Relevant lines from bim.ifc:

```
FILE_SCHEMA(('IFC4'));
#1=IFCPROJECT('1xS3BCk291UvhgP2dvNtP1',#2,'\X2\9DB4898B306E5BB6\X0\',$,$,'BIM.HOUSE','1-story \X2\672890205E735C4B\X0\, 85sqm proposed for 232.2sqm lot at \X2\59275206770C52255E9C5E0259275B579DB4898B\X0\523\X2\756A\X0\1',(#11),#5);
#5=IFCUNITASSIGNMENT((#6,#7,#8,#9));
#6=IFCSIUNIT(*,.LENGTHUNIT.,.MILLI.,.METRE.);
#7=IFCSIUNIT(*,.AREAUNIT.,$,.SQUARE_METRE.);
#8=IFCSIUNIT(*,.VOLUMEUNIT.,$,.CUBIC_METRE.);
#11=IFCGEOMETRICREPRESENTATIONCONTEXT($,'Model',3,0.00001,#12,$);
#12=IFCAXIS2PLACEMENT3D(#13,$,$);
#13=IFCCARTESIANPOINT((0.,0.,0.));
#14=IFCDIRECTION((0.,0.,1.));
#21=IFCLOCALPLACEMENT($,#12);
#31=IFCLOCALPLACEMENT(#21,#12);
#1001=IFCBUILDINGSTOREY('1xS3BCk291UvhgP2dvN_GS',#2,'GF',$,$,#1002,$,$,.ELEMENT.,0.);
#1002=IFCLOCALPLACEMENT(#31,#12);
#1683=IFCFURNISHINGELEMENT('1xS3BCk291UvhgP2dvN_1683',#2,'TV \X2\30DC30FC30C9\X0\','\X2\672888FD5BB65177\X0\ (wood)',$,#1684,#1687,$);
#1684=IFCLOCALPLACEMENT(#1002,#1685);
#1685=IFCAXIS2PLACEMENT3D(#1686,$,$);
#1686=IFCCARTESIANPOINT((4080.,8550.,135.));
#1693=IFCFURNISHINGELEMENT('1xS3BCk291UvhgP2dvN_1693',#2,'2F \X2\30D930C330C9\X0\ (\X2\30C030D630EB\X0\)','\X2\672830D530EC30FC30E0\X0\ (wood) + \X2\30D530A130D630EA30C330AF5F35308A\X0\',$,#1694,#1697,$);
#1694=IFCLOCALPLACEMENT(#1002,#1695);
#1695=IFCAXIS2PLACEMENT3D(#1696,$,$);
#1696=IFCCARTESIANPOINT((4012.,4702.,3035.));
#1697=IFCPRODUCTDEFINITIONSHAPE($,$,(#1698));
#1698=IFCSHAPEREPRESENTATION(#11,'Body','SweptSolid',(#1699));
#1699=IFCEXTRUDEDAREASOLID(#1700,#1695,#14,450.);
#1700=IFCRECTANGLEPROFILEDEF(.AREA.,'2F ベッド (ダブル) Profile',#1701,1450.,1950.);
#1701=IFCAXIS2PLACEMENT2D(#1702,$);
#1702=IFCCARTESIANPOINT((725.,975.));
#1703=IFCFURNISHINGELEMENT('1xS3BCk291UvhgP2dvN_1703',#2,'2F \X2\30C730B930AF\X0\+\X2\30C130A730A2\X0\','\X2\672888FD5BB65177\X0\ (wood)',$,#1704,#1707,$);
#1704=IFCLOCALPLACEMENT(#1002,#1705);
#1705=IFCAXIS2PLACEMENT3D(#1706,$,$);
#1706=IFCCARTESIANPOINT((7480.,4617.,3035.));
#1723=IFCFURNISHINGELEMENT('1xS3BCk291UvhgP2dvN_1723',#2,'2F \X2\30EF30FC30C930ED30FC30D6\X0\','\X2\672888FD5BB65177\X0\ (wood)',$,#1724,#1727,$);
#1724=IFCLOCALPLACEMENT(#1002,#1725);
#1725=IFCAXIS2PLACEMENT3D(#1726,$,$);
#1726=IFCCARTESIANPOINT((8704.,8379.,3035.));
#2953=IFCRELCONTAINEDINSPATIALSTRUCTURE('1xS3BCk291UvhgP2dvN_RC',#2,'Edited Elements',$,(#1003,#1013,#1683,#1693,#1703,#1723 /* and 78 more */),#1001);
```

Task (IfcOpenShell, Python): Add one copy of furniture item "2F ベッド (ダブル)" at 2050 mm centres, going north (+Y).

```python
import numpy as np
import ifcopenshell
import ifcopenshell.api.geometry
import ifcopenshell.api.root
import ifcopenshell.util.element
import ifcopenshell.util.placement
import ifcopenshell.util.unit

model = ifcopenshell.open("bim.ifc")
unit_scale = ifcopenshell.util.unit.calculate_unit_scale(model)


def reuse_history(source, copy):
    """copy_class also copies each property set's owner history, people and application; keep the originals."""
    for rel in copy.IsDefinedBy:
        if rel.is_a("IfcRelDefinesByProperties") and (history := rel.RelatingPropertyDefinition.OwnerHistory):
            rel.RelatingPropertyDefinition.OwnerHistory = source.OwnerHistory
            ifcopenshell.util.element.remove_deep2(model, history)


source = model.by_id(1693)
base = ifcopenshell.util.placement.get_local_placement(source.ObjectPlacement)
step = np.array([0.0, 1.0, 0.0]) * 2.05 / unit_scale

for i in range(1, 2):
    copy = ifcopenshell.api.root.copy_class(model, product=source)
    copy.Representation = ifcopenshell.util.element.copy_deep(
        model, source.Representation, exclude=["IfcGeometricRepresentationContext", "IfcRepresentationMap"]
    )
    reuse_history(source, copy)
    matrix = base.copy()
    matrix[:3, 3] += i * step
    print("added at", matrix[:3, 3].round(3) + 0.0)
    ifcopenshell.api.geometry.edit_object_placement(model, product=copy, matrix=matrix, is_si=False)

model.write("bim_edited.ifc")
```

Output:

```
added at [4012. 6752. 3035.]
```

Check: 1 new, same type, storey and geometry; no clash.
